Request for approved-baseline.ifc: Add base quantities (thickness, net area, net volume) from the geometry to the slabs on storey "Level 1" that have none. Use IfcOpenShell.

First a look at what the model holds.

```python
import ifcopenshell
import ifcopenshell.util.element
import ifcopenshell.util.unit

model = ifcopenshell.open("approved-baseline.ifc")
print(model.schema)
for unit_type in ("LENGTHUNIT", "AREAUNIT", "VOLUMEUNIT"):
    print(unit_type, ifcopenshell.util.unit.calculate_unit_scale(model, unit_type))
storey = next(s for s in model.by_type("IfcBuildingStorey") if s.Name == "Level 1")
slabs = [e for e in ifcopenshell.util.element.get_decomposition(storey) if e.is_a("IfcSlab")]
for e in sorted(slabs, key=lambda e: e.id()):
    print(e.id(), e.is_a(), e.Name, list(ifcopenshell.util.element.get_psets(e, qtos_only=True)), sep=" | ")
```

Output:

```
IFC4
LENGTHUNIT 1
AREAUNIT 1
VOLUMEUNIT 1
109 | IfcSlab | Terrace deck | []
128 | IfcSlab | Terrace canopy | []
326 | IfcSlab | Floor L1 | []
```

```python
import ifcopenshell
import ifcopenshell.api.pset
import ifcopenshell.geom
import ifcopenshell.util.element
import ifcopenshell.util.shape
import ifcopenshell.util.unit

model = ifcopenshell.open("approved-baseline.ifc")
unit_scale = ifcopenshell.util.unit.calculate_unit_scale(model)
area_scale = ifcopenshell.util.unit.calculate_unit_scale(model, "AREAUNIT")
volume_scale = ifcopenshell.util.unit.calculate_unit_scale(model, "VOLUMEUNIT")
settings = ifcopenshell.geom.settings()

storey = next(s for s in model.by_type("IfcBuildingStorey") if s.Name == "Level 1")
slabs = [e for e in ifcopenshell.util.element.get_decomposition(storey) if e.is_a("IfcSlab")]

for e in sorted(slabs, key=lambda e: e.id()):
    if ifcopenshell.util.element.get_psets(e, qtos_only=True, should_inherit=False):
        continue
    # Geometry comes back in metres, in the element's own axes.
    shape = ifcopenshell.geom.create_shape(settings, e)
    values = {
        "Width": ifcopenshell.util.shape.get_z(shape.geometry) / unit_scale,
        "NetArea": ifcopenshell.util.shape.get_footprint_area(shape.geometry) / area_scale,
        "NetVolume": ifcopenshell.util.shape.get_volume(shape.geometry) / volume_scale,
    }
    qto = ifcopenshell.api.pset.add_qto(model, product=e, name="Qto_SlabBaseQuantities")
    ifcopenshell.api.pset.edit_qto(model, qto=qto, properties=values)
    print(e.id(), {k: round(v, 3) for k, v in values.items()})

model.write("approved-baseline-out.ifc")
```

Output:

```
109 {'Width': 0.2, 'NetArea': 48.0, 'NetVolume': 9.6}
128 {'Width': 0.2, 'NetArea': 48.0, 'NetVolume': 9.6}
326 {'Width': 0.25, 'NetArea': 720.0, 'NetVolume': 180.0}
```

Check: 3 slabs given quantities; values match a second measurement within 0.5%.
